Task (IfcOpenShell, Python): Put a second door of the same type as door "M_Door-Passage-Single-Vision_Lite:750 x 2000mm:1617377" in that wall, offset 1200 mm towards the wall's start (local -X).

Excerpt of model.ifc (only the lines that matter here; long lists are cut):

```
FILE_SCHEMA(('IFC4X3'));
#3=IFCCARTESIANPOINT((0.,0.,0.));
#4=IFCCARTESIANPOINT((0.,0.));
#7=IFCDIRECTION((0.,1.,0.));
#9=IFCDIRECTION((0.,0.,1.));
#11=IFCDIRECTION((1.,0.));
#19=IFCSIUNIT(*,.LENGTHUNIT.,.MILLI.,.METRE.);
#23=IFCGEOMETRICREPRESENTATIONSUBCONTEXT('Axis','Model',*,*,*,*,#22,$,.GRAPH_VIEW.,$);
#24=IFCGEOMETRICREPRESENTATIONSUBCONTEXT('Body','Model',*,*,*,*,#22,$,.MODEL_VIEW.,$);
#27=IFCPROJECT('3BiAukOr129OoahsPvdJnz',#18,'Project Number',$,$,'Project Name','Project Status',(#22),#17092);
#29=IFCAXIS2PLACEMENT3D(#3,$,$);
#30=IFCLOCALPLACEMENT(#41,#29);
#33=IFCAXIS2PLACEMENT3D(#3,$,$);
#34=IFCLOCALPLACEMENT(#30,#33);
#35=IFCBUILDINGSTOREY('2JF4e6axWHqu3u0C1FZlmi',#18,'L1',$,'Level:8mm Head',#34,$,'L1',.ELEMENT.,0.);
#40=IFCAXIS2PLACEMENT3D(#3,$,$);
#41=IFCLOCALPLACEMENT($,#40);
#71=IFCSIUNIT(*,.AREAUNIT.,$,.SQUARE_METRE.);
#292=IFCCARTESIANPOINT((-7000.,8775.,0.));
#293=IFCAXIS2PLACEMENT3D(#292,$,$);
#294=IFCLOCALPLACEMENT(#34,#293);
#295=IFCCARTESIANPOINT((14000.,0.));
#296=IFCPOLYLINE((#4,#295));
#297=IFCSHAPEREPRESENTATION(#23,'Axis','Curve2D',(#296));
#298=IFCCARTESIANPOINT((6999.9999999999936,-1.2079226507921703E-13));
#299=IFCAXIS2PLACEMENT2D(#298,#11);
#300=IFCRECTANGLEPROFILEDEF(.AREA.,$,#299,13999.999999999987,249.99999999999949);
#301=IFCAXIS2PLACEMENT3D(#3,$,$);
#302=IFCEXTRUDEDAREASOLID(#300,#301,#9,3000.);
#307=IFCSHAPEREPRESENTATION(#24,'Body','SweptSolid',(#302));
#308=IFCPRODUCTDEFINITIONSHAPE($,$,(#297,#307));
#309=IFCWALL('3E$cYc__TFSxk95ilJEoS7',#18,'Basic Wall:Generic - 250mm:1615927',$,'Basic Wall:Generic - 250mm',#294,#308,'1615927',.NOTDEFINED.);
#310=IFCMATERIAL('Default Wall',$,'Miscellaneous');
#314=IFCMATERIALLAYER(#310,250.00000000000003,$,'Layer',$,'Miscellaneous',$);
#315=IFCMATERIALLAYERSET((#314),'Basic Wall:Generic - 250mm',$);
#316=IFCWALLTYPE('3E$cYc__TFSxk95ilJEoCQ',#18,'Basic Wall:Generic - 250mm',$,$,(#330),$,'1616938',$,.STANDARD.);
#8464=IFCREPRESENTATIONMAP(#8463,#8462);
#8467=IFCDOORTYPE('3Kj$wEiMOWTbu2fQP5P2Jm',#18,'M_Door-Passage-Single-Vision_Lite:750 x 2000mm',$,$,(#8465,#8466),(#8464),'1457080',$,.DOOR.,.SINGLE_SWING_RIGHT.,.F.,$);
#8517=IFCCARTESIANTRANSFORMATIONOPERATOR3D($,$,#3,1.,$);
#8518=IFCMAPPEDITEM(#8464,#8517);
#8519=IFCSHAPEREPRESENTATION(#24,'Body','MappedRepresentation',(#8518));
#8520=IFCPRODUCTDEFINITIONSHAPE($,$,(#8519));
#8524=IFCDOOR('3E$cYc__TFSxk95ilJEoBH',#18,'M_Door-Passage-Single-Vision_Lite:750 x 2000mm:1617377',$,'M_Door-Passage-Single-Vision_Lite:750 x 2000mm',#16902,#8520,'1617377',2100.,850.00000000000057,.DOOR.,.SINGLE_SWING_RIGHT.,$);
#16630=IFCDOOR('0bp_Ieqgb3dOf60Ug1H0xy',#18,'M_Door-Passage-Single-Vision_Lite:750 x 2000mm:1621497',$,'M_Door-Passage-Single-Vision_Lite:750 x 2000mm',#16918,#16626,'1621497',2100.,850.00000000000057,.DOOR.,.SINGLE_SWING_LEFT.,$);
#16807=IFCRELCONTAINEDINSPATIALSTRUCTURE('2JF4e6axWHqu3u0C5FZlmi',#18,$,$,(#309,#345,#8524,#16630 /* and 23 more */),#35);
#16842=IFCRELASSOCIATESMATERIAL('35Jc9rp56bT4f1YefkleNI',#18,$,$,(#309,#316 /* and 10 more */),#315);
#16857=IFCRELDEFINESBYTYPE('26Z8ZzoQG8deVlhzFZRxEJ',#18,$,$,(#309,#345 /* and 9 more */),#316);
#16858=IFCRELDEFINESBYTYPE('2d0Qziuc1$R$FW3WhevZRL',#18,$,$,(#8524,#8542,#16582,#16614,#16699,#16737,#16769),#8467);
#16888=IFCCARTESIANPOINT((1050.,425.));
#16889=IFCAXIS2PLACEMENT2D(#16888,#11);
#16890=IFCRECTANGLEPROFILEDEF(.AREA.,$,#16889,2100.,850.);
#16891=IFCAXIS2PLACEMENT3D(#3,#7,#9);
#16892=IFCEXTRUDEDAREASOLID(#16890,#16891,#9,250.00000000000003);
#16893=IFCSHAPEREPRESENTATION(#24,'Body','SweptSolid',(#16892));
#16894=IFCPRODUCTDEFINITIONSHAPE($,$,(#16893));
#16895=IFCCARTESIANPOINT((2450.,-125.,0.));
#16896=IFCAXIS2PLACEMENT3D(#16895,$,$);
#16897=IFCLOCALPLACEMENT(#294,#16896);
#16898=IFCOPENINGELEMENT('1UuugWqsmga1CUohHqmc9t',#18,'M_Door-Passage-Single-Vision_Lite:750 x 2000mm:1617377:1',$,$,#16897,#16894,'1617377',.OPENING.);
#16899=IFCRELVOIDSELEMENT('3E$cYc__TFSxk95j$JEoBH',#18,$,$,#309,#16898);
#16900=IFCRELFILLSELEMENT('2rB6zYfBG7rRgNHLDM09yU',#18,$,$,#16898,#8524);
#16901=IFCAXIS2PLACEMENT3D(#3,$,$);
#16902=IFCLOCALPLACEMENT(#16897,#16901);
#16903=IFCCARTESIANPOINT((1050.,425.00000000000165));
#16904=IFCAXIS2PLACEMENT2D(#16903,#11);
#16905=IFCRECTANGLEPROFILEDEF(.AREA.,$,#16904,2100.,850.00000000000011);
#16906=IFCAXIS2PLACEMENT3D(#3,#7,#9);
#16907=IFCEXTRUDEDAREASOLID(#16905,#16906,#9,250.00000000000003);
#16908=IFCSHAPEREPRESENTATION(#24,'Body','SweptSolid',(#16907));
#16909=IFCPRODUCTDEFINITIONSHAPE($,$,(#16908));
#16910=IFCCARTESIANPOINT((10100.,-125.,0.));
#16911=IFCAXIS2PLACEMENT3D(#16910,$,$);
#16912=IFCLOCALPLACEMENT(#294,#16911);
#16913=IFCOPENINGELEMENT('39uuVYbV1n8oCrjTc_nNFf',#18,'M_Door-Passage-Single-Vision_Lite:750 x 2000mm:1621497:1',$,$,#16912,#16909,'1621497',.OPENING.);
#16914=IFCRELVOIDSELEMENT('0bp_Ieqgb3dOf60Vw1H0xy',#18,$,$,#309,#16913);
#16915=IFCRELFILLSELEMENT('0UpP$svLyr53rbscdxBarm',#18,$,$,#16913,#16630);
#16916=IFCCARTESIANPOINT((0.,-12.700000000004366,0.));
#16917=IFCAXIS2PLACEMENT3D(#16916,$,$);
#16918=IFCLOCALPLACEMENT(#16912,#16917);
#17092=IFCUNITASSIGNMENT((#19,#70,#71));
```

```python
import ifcopenshell
import ifcopenshell.api.feature
import ifcopenshell.api.geometry
import ifcopenshell.api.root
import ifcopenshell.geom
import ifcopenshell.util.element
import ifcopenshell.util.placement
import ifcopenshell.util.shape
import ifcopenshell.util.unit

model = ifcopenshell.open("model.ifc")
unit_scale = ifcopenshell.util.unit.calculate_unit_scale(model)
settings = ifcopenshell.geom.settings()


def volume(element):
    """Net volume in cubic metres, openings subtracted."""
    shape = ifcopenshell.geom.create_shape(settings, element)
    return ifcopenshell.util.shape.get_volume(shape.geometry)


def reuse_history(source, copy):
    """copy_class also copies each property set's owner history, people and application; keep the originals."""
    for rel in copy.IsDefinedBy:
        if rel.is_a("IfcRelDefinesByProperties") and (history := rel.RelatingPropertyDefinition.OwnerHistory):
            rel.RelatingPropertyDefinition.OwnerHistory = source.OwnerHistory
            ifcopenshell.util.element.remove_deep2(model, history)


door = model.by_guid("3E$cYc__TFSxk95ilJEoBH")
opening = door.FillsVoids[0].RelatingOpeningElement
wall = opening.VoidsElements[0].RelatingBuildingElement
before = volume(wall)
shift = ifcopenshell.util.placement.get_local_placement(wall.ObjectPlacement)[:3, 0] * -1.2 / unit_scale

# copy_class copies the void relationship, type, container and properties, but no geometry.
new_opening = ifcopenshell.api.root.copy_class(model, product=opening)
new_opening.Representation = ifcopenshell.util.element.copy_deep(
    model, opening.Representation, exclude=["IfcGeometricRepresentationContext", "IfcRepresentationMap"]
)
new_opening.Name = "M_Door-Passage-Single-Vision_Lite:750 x 2000mm"
new_opening.Tag = None
new_door = ifcopenshell.api.root.copy_class(model, product=door)
new_door.Representation = ifcopenshell.util.element.copy_deep(
    model, door.Representation, exclude=["IfcGeometricRepresentationContext", "IfcRepresentationMap"]
)
new_door.Name = "M_Door-Passage-Single-Vision_Lite:750 x 2000mm"
new_door.Tag = None
reuse_history(door, new_door)
ifcopenshell.api.feature.add_filling(model, opening=new_opening, element=new_door)

for old, new in ((opening, new_opening), (door, new_door)):
    matrix = ifcopenshell.util.placement.get_local_placement(old.ObjectPlacement)
    matrix[:3, 3] += shift
    ifcopenshell.api.geometry.edit_object_placement(model, product=new, matrix=matrix, is_si=False)

after = volume(wall)

print(f"wall volume {before:.3f} -> {after:.3f} m3")

model.write("model-out.ifc")
```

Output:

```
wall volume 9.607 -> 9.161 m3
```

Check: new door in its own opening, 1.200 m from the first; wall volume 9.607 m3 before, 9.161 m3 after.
